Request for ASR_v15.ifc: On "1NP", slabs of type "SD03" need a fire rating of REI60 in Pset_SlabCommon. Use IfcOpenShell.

First a look at what the model holds.

```python
import ifcopenshell
import ifcopenshell.util.element

model = ifcopenshell.open("ASR_v15.ifc")
print(model.schema)
storey = next(s for s in model.by_type("IfcBuildingStorey") if s.Name == "1NP")
slabs = [e for e in ifcopenshell.util.element.get_decomposition(storey) if e.is_a("IfcSlab")]
seen = {}
for e in slabs:
    element_type = ifcopenshell.util.element.get_type(e)
    key = (element_type.Name if element_type != e and element_type else None, ifcopenshell.util.element.get_pset(e, "Pset_SlabCommon", "FireRating"))
    seen[key] = seen.get(key, 0) + 1
for (name, value), count in sorted(seen.items(), key=str):
    print(count, "x", name, "|", value)
```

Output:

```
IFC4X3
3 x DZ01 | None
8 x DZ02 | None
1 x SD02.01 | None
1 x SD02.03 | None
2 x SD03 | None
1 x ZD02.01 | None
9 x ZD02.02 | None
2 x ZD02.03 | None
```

```python
import ifcopenshell
import ifcopenshell.api.pset
import ifcopenshell.util.element

model = ifcopenshell.open("ASR_v15.ifc")

storey = next(s for s in model.by_type("IfcBuildingStorey") if s.Name == "1NP")
slabs = [e for e in ifcopenshell.util.element.get_decomposition(storey) if e.is_a("IfcSlab")]

count = 0
for e in slabs:
    element_type = ifcopenshell.util.element.get_type(e)
    if element_type in (None, e) or element_type.Name != "SD03":
        continue
    # add_pset returns the element's existing set when there is one.
    pset = ifcopenshell.api.pset.add_pset(model, product=e, name="Pset_SlabCommon")
    ifcopenshell.api.pset.edit_pset(model, pset=pset, properties={"FireRating": "REI60"})
    count += 1

print(count, "slabs updated")

model.write("ASR_v15-out.ifc")
```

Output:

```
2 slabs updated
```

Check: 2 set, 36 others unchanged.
